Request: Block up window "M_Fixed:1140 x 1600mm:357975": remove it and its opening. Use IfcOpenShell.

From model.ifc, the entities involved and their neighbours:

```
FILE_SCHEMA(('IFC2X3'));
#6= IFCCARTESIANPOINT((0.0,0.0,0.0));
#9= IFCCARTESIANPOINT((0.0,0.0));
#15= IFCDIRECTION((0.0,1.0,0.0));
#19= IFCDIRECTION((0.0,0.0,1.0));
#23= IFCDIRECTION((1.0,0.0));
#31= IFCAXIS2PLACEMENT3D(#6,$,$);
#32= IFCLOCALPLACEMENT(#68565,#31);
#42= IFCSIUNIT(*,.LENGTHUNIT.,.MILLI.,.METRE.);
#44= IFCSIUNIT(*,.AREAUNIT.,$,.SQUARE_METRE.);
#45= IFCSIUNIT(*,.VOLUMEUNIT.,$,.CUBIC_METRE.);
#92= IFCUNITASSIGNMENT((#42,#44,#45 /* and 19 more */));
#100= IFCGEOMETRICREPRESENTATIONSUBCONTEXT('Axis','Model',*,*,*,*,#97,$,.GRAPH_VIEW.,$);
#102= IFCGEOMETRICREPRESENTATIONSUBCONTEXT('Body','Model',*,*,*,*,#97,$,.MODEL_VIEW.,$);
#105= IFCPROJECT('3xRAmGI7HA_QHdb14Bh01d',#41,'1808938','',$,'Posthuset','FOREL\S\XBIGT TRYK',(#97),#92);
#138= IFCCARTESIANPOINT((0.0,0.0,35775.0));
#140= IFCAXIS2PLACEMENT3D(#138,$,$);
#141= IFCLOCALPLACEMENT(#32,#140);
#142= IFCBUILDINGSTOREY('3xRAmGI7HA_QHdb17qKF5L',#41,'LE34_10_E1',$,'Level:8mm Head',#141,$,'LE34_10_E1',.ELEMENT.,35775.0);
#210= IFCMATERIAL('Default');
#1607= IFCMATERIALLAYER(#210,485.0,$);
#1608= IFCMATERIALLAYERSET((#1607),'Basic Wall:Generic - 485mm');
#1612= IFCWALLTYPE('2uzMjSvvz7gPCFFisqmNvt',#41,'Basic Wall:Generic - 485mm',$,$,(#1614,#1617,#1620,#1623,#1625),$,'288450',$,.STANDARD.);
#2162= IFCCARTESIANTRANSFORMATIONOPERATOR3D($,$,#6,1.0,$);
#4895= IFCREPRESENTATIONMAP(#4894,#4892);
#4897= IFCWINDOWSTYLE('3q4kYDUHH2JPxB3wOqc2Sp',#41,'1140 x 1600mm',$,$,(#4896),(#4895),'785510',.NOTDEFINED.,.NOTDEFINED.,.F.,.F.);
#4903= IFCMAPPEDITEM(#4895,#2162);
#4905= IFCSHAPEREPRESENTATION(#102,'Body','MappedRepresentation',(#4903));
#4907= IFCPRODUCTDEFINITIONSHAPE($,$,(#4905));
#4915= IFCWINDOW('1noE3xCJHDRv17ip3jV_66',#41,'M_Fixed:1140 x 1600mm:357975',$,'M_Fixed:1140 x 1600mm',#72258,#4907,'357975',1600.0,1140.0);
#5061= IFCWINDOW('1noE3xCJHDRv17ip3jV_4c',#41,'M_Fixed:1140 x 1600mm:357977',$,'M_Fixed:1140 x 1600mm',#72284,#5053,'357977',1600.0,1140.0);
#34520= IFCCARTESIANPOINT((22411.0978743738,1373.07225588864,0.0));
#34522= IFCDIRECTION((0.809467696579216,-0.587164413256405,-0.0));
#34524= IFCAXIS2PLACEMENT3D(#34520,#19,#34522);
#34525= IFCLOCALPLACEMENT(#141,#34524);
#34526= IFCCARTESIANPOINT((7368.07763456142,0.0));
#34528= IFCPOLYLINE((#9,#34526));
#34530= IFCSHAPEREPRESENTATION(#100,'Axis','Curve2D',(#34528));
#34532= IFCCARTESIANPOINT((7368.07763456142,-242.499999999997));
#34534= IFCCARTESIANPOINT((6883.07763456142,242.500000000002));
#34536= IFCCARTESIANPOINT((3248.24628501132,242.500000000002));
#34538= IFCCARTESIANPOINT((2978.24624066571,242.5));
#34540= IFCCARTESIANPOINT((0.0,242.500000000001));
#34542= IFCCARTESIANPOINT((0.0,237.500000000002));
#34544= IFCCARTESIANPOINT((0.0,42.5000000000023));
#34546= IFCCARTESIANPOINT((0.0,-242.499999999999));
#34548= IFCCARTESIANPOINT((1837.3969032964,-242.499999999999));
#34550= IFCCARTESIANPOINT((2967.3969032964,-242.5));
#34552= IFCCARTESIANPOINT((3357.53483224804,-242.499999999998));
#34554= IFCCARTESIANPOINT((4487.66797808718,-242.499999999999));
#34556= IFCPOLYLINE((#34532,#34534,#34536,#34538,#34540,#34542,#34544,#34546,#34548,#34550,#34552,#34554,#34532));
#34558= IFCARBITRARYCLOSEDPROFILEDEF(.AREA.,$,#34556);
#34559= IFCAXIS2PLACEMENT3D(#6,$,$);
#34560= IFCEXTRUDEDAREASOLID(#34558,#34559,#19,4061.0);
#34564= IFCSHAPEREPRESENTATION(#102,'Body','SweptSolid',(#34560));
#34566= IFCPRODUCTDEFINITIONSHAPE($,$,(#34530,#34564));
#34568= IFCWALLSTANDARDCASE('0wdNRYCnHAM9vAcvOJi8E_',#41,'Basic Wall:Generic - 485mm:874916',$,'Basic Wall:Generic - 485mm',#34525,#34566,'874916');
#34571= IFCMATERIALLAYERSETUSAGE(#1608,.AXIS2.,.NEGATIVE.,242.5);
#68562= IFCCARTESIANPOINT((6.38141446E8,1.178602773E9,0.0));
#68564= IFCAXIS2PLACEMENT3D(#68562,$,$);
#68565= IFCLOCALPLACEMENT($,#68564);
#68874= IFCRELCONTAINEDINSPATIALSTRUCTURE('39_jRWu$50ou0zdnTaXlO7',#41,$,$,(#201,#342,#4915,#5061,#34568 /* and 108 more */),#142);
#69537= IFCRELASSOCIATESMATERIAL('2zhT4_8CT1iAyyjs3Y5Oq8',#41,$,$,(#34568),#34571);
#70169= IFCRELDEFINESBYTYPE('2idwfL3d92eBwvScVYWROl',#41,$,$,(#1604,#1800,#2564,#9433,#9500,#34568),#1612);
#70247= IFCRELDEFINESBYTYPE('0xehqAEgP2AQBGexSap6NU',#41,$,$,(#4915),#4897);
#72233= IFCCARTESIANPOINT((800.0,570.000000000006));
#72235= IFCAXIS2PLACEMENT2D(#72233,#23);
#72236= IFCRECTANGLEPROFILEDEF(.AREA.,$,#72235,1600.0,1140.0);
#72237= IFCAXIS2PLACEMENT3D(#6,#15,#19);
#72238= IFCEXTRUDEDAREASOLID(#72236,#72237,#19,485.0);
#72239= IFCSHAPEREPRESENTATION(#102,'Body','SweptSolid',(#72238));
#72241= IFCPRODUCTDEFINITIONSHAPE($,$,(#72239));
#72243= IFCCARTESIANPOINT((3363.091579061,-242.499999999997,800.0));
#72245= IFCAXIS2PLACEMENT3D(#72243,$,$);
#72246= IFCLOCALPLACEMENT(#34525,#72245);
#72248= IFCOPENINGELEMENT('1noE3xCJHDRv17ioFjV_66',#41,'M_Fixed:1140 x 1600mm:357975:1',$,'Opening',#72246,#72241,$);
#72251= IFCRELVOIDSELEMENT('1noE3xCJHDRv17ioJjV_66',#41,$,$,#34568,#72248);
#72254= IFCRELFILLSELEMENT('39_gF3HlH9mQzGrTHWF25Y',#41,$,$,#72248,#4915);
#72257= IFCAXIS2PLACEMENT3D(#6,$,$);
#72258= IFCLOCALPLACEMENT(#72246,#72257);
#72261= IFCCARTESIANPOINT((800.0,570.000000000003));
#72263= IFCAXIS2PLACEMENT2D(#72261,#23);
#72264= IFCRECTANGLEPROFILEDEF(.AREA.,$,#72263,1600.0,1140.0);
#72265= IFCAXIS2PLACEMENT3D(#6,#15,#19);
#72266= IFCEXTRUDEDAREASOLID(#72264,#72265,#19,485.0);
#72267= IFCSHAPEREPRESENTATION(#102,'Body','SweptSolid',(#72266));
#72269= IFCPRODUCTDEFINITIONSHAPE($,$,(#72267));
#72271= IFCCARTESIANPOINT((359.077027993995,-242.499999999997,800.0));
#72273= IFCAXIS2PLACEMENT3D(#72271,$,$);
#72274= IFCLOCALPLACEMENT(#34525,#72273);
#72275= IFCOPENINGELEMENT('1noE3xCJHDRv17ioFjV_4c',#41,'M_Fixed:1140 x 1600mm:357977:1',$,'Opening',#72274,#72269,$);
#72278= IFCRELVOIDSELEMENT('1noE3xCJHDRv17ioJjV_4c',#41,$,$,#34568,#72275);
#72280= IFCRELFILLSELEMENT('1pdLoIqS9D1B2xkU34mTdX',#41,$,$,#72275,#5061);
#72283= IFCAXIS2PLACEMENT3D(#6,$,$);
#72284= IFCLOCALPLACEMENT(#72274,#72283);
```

```python
import ifcopenshell
import ifcopenshell.api.feature
import ifcopenshell.api.root
import ifcopenshell.geom
import ifcopenshell.util.shape

model = ifcopenshell.open("model.ifc")
settings = ifcopenshell.geom.settings()


def volume(element):
    """Net volume in cubic metres, openings subtracted."""
    shape = ifcopenshell.geom.create_shape(settings, element)
    return ifcopenshell.util.shape.get_volume(shape.geometry)


window = model.by_guid("1noE3xCJHDRv17ip3jV_66")
opening = window.FillsVoids[0].RelatingOpeningElement
wall = opening.VoidsElements[0].RelatingBuildingElement
before = volume(wall)

ifcopenshell.api.root.remove_product(model, product=window)
ifcopenshell.api.feature.remove_feature(model, feature=opening)

after = volume(wall)

print(f"wall volume {before:.3f} -> {after:.3f} m3")

model.write("model_updated.ifc")
```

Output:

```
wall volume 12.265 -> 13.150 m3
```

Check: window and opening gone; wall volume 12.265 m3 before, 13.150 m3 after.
